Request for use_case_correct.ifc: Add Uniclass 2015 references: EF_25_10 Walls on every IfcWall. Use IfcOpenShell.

First a look at what the model holds.

```python
import ifcopenshell

model = ifcopenshell.open("use_case_correct.ifc")
print(model.schema)
print("classifications:", [c.Name for c in model.by_type("IfcClassification")])
for ifc_class in ("IfcDoor", "IfcRoof", "IfcStair", "IfcWall", "IfcWindow"):
    print(ifc_class, len(model.by_type(ifc_class)))
```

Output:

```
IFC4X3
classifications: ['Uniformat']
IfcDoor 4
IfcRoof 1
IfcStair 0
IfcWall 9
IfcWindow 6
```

```python
import ifcopenshell
import ifcopenshell.api.classification

model = ifcopenshell.open("use_case_correct.ifc")

system = ifcopenshell.api.classification.add_classification(model, classification="Uniclass 2015")

codes = {
    "IfcWall": ("EF_25_10", "Walls"),
}
for ifc_class, (code, name) in codes.items():
    products = model.by_type(ifc_class)
    ifcopenshell.api.classification.add_reference(
        model, products=products, classification=system, identification=code, name=name
    )
    print(code, len(products))

model.write("use_case_correct_edited.ifc")
```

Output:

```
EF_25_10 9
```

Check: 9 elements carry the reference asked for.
